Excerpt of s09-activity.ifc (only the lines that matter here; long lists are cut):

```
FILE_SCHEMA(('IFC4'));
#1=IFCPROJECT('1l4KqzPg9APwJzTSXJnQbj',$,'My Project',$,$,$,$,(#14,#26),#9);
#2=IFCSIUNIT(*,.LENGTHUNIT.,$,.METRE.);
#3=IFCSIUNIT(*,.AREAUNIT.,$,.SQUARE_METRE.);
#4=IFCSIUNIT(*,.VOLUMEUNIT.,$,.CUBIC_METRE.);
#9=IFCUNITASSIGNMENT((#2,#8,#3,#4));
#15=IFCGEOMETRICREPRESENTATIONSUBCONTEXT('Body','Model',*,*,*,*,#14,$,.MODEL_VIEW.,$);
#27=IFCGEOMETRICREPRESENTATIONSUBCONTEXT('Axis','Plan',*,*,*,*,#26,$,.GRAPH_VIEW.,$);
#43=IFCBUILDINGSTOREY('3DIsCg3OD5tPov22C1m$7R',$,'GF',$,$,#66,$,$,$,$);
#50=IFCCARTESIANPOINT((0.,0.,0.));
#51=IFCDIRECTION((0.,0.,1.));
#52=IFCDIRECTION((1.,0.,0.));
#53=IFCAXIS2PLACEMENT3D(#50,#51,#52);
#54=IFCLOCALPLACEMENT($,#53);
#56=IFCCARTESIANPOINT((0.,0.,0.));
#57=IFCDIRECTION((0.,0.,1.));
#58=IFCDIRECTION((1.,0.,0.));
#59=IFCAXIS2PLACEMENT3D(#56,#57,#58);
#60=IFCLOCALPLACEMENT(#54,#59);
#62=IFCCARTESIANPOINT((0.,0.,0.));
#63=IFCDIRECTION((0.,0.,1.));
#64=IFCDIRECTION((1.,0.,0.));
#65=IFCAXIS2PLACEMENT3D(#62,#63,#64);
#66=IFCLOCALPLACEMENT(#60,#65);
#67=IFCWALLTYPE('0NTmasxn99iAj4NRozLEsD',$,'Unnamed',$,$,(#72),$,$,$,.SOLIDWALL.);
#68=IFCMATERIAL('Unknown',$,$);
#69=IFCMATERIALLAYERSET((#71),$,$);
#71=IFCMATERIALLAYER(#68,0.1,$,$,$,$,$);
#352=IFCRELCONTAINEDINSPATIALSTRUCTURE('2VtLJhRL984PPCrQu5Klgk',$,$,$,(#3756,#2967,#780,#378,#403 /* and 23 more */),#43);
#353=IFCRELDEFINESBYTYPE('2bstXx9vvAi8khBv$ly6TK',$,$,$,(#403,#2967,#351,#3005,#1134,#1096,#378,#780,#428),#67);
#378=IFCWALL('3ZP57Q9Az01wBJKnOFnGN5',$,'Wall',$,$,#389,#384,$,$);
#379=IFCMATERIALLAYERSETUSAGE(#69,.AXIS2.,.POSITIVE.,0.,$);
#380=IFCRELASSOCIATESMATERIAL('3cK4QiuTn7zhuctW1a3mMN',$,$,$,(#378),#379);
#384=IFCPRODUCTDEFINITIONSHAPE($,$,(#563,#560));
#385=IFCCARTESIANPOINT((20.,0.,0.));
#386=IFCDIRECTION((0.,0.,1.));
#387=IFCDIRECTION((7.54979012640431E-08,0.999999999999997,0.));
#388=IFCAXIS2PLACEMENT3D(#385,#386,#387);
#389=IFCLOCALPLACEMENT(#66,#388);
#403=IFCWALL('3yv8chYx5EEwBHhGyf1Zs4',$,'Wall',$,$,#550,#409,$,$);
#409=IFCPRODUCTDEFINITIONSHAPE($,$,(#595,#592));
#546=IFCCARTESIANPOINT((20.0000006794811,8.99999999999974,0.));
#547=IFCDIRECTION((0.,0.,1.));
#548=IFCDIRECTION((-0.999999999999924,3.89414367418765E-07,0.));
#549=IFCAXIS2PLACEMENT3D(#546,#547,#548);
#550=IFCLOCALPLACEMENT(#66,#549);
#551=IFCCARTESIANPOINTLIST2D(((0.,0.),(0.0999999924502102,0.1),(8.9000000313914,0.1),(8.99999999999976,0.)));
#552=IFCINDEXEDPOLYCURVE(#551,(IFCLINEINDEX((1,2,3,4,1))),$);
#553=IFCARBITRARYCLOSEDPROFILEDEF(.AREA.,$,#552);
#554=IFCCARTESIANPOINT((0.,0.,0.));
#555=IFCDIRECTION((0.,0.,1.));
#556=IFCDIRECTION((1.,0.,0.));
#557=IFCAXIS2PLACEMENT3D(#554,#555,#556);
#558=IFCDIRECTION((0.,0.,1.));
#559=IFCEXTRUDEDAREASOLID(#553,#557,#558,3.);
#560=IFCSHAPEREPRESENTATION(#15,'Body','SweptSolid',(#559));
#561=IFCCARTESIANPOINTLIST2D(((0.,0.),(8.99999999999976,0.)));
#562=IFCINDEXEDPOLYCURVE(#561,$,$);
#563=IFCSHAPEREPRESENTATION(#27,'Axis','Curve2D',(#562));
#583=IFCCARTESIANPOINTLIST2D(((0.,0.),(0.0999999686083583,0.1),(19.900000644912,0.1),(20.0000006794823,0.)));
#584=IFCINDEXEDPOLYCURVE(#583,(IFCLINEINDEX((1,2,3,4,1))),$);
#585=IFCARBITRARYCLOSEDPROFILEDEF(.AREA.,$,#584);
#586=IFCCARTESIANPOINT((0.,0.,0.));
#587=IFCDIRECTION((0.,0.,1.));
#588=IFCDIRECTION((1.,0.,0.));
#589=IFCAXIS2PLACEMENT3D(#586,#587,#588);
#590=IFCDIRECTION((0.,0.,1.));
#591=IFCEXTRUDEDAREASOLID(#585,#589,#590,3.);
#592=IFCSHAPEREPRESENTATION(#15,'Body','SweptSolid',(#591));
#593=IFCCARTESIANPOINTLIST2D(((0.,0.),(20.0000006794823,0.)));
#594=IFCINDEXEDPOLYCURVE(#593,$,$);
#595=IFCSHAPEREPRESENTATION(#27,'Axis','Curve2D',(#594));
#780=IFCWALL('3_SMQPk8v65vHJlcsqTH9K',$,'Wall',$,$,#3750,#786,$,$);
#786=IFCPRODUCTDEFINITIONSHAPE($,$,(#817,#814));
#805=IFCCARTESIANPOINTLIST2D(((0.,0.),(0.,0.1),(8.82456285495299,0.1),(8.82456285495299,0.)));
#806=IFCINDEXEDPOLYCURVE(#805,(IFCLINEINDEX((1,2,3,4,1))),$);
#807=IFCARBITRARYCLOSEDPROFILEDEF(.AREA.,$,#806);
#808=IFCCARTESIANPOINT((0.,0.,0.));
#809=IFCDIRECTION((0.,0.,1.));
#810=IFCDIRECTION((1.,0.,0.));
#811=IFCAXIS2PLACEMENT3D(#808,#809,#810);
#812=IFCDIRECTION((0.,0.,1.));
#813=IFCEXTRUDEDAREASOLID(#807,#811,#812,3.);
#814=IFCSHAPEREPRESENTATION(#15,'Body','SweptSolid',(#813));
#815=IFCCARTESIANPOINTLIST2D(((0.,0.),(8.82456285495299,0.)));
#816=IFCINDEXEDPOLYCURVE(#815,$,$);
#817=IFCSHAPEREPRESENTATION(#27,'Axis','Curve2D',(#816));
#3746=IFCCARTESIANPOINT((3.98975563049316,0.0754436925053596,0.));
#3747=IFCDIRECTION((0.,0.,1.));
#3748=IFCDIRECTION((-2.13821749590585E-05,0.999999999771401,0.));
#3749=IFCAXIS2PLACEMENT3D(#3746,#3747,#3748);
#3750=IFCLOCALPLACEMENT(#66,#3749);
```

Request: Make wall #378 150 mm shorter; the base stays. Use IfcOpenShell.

```python
import ifcopenshell
import ifcopenshell.geom
import ifcopenshell.util.representation
import ifcopenshell.util.shape
import ifcopenshell.util.unit

model = ifcopenshell.open("s09-activity.ifc")
unit_scale = ifcopenshell.util.unit.calculate_unit_scale(model)
settings = ifcopenshell.geom.settings()


def volume(element):
    """Net volume in cubic metres, openings subtracted."""
    shape = ifcopenshell.geom.create_shape(settings, element)
    return ifcopenshell.util.shape.get_volume(shape.geometry)


wall = model.by_guid("3ZP57Q9Az01wBJKnOFnGN5")
before = volume(wall)

body = ifcopenshell.util.representation.get_representation(wall, "Model", "Body")
solid = body.Items[0]
old_height = solid.Depth
solid.Depth -= 0.15 / unit_scale
after = volume(wall)

print(f"height {old_height:g} -> {solid.Depth:g}, volume {before:.3f} -> {after:.3f} m3")

model.write("s09-activity-out.ifc")
```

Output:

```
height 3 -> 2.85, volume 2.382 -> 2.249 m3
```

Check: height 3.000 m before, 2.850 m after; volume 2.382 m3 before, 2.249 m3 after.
